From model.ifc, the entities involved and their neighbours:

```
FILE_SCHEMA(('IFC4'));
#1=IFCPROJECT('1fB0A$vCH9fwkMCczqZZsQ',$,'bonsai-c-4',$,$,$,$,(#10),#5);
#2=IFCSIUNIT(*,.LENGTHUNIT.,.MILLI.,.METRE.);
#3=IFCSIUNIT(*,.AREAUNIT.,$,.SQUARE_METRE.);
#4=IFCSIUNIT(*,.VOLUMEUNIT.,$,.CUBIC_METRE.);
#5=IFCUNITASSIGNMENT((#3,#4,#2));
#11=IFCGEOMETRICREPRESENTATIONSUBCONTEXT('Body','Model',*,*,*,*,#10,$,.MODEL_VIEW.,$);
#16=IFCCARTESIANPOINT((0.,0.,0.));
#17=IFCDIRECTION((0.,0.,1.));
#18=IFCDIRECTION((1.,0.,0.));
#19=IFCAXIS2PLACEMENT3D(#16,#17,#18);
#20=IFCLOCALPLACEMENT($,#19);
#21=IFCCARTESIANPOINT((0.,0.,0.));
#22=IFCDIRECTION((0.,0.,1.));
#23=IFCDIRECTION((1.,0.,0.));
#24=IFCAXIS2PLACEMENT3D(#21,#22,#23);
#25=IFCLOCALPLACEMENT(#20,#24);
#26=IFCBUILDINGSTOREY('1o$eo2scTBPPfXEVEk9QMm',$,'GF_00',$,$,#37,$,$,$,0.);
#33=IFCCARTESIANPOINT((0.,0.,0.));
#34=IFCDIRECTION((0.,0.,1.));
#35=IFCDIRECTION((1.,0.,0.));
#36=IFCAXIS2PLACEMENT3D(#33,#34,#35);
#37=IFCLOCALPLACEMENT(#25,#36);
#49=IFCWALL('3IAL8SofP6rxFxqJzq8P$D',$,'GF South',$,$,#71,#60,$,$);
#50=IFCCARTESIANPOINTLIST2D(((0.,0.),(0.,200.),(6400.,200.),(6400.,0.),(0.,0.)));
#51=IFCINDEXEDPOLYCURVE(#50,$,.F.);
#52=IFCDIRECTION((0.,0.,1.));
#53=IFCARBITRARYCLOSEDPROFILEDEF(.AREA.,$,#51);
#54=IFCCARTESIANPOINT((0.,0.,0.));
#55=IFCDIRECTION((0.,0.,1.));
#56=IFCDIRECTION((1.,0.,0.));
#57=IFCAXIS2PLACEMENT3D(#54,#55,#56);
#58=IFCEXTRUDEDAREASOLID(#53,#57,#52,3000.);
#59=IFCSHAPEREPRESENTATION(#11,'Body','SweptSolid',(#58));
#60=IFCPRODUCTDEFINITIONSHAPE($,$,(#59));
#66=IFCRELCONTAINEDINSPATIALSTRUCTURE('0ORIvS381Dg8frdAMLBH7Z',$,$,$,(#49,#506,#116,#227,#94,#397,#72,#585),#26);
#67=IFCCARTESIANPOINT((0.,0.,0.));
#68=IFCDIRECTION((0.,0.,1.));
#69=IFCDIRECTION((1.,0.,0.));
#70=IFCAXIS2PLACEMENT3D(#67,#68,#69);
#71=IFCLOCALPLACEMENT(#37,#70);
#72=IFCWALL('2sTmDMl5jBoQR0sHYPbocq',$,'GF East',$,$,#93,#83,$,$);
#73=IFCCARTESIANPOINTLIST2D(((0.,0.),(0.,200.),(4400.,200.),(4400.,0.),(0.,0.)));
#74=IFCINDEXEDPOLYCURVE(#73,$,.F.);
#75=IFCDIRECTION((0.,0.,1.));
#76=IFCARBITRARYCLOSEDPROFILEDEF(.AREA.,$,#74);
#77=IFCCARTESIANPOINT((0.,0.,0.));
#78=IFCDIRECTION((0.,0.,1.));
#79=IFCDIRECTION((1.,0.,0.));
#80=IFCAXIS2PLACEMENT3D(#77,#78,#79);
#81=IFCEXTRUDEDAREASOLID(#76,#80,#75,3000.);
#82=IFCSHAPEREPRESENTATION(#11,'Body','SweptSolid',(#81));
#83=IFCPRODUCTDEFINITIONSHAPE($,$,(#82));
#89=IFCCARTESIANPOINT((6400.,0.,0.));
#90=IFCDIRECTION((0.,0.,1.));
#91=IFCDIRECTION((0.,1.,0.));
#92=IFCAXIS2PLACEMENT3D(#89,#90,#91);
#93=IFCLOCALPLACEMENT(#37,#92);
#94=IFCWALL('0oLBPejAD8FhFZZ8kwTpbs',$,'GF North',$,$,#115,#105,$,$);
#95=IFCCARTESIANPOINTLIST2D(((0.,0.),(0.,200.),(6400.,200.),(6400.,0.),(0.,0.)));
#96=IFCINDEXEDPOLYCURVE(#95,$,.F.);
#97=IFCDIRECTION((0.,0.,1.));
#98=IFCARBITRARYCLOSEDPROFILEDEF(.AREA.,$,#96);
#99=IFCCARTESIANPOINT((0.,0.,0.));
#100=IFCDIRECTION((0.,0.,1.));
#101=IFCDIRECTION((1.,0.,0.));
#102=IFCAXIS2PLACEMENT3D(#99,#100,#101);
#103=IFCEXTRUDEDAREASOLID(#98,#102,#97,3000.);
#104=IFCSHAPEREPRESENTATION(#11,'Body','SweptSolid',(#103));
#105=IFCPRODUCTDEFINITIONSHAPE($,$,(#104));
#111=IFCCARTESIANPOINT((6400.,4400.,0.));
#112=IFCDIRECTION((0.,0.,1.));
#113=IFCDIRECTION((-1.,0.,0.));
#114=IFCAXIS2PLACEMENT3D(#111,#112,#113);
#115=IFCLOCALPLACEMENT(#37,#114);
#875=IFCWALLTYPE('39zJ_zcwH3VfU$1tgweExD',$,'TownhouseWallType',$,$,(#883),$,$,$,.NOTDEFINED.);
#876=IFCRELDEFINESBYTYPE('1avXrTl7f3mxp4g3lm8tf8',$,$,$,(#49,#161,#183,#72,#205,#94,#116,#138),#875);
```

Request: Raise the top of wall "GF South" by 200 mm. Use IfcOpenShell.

```python
import ifcopenshell
import ifcopenshell.geom
import ifcopenshell.util.representation
import ifcopenshell.util.shape
import ifcopenshell.util.unit

model = ifcopenshell.open("model.ifc")
unit_scale = ifcopenshell.util.unit.calculate_unit_scale(model)
settings = ifcopenshell.geom.settings()


def volume(element):
    """Net volume in cubic metres, openings subtracted."""
    shape = ifcopenshell.geom.create_shape(settings, element)
    return ifcopenshell.util.shape.get_volume(shape.geometry)


wall = model.by_guid("3IAL8SofP6rxFxqJzq8P$D")
before = volume(wall)

body = ifcopenshell.util.representation.get_representation(wall, "Model", "Body")
solid = body.Items[0]
old_height = solid.Depth
solid.Depth += 0.2 / unit_scale
after = volume(wall)

print(f"height {old_height:g} -> {solid.Depth:g}, volume {before:.3f} -> {after:.3f} m3")

model.write("model_v2.ifc")
```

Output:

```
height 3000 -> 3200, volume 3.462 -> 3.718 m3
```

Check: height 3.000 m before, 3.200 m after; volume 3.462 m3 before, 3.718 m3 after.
